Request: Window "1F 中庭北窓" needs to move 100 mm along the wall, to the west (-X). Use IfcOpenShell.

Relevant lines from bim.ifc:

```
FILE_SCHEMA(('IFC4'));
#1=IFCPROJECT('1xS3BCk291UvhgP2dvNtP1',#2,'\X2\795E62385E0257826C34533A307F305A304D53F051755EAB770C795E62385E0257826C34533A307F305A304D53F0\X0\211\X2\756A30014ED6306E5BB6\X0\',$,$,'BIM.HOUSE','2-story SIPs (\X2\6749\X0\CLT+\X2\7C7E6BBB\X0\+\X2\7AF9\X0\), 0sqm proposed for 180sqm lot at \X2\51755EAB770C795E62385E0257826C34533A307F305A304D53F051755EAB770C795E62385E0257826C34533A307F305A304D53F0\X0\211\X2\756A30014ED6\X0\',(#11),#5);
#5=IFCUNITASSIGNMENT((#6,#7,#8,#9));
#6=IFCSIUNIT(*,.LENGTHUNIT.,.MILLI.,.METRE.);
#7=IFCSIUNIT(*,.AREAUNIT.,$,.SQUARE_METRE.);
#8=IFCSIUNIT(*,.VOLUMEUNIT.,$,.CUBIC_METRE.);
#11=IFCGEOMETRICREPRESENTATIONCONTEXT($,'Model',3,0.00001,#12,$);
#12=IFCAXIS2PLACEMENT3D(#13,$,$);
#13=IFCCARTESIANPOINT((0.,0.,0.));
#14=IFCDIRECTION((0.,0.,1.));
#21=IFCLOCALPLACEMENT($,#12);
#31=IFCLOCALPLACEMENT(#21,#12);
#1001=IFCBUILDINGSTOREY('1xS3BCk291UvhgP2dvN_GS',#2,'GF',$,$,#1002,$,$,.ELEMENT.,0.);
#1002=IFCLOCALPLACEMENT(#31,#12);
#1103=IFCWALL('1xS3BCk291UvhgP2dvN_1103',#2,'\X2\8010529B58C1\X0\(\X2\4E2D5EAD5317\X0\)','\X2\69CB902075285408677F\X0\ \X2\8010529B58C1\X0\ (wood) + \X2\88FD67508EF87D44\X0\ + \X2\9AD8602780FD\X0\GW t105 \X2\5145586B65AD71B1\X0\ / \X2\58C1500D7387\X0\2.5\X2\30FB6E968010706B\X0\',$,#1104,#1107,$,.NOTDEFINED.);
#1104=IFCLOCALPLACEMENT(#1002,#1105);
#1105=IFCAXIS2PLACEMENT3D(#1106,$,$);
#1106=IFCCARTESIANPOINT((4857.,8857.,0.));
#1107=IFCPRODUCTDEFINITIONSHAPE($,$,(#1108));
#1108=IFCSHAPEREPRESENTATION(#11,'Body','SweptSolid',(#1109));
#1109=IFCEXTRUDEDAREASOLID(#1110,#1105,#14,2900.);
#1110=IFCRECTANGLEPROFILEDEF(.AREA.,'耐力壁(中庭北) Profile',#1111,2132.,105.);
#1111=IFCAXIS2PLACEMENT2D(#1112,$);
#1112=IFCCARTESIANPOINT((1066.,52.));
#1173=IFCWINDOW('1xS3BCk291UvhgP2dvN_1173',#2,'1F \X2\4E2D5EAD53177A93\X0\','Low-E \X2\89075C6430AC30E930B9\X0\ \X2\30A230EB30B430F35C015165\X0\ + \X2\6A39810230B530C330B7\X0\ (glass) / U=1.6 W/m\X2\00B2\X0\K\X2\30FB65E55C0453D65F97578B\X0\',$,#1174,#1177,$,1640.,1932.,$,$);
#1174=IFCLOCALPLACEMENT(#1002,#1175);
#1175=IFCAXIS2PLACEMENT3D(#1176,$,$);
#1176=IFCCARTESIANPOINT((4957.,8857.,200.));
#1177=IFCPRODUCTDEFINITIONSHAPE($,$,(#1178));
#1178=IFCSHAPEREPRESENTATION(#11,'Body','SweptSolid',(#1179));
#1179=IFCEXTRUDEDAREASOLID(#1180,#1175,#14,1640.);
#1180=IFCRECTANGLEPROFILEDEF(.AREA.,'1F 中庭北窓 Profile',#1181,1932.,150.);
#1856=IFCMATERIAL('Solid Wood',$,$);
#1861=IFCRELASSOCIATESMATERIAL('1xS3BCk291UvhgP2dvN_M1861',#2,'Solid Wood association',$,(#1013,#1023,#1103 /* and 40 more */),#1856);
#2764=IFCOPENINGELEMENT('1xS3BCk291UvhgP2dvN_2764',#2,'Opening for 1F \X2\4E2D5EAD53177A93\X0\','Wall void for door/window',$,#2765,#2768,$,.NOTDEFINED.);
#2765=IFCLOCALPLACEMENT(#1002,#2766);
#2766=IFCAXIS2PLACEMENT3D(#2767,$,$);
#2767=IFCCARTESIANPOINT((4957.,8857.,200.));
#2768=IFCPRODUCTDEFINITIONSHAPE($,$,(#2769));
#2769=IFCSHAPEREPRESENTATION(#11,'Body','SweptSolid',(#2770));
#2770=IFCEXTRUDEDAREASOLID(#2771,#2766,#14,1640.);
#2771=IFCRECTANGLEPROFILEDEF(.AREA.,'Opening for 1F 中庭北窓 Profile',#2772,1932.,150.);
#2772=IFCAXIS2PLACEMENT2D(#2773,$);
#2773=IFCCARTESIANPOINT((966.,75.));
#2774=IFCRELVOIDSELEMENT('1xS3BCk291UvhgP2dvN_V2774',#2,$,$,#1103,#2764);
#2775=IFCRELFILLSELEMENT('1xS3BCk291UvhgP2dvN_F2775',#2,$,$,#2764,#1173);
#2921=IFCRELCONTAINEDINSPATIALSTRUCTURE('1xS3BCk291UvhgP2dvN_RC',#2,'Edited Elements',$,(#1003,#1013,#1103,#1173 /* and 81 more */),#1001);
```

```python
import ifcopenshell
import ifcopenshell.api.geometry
import ifcopenshell.util.placement
import ifcopenshell.util.unit

model = ifcopenshell.open("bim.ifc")
unit_scale = ifcopenshell.util.unit.calculate_unit_scale(model)

window = model.by_guid("1xS3BCk291UvhgP2dvN_1173")
opening = window.FillsVoids[0].RelatingOpeningElement
wall = opening.VoidsElements[0].RelatingBuildingElement

wall_matrix = ifcopenshell.util.placement.get_local_placement(wall.ObjectPlacement)
shift = wall_matrix[:3, 0] * -0.1 / unit_scale
before = ifcopenshell.util.placement.get_local_placement(window.ObjectPlacement)[:3, 3].copy()

# The window is not placed relative to its opening, so move both.
for product in (opening, window):
    matrix = ifcopenshell.util.placement.get_local_placement(product.ObjectPlacement)
    matrix[:3, 3] += shift
    ifcopenshell.api.geometry.edit_object_placement(model, product=product, matrix=matrix, is_si=False)

after = ifcopenshell.util.placement.get_local_placement(window.ObjectPlacement)[:3, 3]
print("window moved by", (after - before).round(3) + 0.0)

model.write("bim_edited.ifc")
```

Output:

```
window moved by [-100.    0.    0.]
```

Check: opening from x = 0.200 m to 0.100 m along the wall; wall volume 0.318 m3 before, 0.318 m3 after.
